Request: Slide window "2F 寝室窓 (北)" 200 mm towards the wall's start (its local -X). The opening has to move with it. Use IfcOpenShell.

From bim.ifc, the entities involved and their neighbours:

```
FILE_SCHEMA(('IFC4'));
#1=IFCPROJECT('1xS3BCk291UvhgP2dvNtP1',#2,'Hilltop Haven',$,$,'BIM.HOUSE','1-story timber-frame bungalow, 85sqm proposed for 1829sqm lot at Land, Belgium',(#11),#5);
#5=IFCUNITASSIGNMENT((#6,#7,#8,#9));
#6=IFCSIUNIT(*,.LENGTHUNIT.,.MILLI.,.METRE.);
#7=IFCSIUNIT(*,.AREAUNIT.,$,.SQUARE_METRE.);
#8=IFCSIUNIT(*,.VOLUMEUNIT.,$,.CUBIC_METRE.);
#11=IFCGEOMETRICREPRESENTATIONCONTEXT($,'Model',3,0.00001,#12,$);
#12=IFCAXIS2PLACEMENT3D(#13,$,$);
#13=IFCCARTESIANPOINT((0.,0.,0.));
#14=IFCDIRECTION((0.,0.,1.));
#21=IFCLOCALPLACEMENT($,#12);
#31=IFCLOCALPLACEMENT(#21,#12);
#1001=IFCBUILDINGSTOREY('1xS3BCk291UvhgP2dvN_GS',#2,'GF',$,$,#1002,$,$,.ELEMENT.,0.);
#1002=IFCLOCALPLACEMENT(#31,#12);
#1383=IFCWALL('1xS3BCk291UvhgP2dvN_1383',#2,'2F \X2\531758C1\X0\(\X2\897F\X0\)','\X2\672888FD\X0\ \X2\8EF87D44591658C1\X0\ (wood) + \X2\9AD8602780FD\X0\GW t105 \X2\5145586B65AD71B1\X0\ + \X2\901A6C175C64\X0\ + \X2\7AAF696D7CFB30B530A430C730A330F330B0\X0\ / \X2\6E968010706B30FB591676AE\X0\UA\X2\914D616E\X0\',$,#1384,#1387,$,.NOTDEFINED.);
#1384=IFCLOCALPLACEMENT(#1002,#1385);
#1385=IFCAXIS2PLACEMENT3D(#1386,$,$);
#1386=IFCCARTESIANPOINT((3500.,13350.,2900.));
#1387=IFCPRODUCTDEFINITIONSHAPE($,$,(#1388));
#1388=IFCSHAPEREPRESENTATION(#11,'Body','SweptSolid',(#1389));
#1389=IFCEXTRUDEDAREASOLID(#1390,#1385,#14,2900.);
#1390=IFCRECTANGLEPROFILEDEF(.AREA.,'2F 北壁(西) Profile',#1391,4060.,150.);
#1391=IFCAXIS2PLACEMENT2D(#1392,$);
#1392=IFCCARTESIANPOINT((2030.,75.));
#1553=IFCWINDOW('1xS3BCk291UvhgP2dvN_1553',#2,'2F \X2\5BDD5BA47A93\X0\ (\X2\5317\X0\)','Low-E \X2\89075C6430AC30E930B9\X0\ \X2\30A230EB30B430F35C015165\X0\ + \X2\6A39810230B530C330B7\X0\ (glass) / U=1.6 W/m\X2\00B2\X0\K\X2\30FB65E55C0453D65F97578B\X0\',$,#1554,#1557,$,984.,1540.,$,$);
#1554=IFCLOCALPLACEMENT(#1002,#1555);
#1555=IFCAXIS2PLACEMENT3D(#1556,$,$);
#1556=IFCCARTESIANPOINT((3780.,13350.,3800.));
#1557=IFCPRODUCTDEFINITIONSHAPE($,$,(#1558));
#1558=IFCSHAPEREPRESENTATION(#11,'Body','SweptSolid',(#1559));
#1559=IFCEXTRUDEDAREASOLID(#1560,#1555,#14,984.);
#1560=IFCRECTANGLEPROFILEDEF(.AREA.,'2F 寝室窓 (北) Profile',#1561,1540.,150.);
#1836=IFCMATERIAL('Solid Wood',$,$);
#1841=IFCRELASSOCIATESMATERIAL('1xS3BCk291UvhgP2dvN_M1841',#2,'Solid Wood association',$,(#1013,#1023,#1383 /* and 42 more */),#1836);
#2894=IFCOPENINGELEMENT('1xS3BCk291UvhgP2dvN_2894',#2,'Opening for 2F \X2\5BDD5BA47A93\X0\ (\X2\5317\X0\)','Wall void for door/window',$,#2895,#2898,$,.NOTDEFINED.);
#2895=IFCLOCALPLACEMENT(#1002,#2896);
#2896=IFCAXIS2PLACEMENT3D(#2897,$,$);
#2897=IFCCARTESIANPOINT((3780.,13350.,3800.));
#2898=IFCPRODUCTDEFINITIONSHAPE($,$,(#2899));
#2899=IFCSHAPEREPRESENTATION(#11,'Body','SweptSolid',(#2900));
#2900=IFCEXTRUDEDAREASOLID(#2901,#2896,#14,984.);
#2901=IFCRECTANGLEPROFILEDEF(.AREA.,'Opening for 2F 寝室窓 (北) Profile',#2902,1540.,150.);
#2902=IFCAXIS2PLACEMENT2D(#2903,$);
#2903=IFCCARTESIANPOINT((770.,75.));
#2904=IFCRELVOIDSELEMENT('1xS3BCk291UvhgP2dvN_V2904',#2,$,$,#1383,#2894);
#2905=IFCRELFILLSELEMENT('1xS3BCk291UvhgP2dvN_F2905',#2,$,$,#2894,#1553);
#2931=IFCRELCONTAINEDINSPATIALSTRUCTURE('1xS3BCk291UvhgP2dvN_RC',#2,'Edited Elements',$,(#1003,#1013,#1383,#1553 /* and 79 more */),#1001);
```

```python
import ifcopenshell
import ifcopenshell.api.geometry
import ifcopenshell.util.placement
import ifcopenshell.util.unit

model = ifcopenshell.open("bim.ifc")
unit_scale = ifcopenshell.util.unit.calculate_unit_scale(model)

window = model.by_guid("1xS3BCk291UvhgP2dvN_1553")
opening = window.FillsVoids[0].RelatingOpeningElement
wall = opening.VoidsElements[0].RelatingBuildingElement

wall_matrix = ifcopenshell.util.placement.get_local_placement(wall.ObjectPlacement)
shift = wall_matrix[:3, 0] * -0.2 / unit_scale
before = ifcopenshell.util.placement.get_local_placement(window.ObjectPlacement)[:3, 3].copy()

# The window is not placed relative to its opening, so move both.
for product in (opening, window):
    matrix = ifcopenshell.util.placement.get_local_placement(product.ObjectPlacement)
    matrix[:3, 3] += shift
    ifcopenshell.api.geometry.edit_object_placement(model, product=product, matrix=matrix, is_si=False)

after = ifcopenshell.util.placement.get_local_placement(window.ObjectPlacement)[:3, 3]
print("window moved by", (after - before).round(3) + 0.0)

model.write("bim_rev.ifc")
```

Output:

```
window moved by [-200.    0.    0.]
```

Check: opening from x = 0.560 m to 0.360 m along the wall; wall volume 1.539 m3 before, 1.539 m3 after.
